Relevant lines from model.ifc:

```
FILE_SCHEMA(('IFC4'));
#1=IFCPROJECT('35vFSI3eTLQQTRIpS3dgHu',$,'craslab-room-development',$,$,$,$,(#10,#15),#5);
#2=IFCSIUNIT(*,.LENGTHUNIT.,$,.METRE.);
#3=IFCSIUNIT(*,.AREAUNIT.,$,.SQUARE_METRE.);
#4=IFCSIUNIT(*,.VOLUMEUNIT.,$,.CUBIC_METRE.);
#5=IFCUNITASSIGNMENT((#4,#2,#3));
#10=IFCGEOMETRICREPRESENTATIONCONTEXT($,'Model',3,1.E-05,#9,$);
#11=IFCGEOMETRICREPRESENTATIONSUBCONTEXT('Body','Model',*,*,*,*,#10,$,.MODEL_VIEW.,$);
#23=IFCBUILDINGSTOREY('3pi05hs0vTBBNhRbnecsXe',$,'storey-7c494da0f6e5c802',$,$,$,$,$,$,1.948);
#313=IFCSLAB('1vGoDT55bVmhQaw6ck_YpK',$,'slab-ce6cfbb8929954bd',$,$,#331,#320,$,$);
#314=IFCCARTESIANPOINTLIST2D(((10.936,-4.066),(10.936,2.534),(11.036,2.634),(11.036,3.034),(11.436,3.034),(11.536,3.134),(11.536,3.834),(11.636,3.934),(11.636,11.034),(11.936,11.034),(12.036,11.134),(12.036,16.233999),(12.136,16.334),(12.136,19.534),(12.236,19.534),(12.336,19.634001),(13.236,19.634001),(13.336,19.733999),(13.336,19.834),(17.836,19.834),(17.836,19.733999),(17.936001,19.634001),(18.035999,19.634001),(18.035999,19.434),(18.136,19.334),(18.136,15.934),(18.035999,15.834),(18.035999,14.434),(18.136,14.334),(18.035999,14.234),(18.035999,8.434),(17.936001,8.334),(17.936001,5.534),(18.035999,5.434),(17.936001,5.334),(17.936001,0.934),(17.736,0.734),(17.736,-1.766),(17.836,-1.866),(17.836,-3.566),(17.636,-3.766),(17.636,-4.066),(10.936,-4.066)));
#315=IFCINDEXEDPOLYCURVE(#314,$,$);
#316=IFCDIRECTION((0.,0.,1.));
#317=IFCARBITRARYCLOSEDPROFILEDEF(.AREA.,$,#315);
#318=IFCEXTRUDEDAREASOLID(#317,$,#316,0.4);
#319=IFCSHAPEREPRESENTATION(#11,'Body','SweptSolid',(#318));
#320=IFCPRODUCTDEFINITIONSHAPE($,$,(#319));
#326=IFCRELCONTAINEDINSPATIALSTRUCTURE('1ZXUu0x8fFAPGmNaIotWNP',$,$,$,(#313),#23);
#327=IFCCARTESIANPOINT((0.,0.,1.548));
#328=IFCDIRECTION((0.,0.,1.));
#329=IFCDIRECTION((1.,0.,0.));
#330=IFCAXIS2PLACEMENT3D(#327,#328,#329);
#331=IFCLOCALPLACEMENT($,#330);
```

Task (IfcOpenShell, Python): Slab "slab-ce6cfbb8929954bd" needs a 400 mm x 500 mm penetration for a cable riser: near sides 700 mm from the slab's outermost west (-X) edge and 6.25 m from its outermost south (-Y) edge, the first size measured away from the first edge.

```python
import numpy as np
import ifcopenshell
import ifcopenshell.api.feature
import ifcopenshell.api.geometry
import ifcopenshell.api.root
import ifcopenshell.geom
import ifcopenshell.util.placement
import ifcopenshell.util.representation
import ifcopenshell.util.shape
import ifcopenshell.util.unit

model = ifcopenshell.open("model.ifc")
unit_scale = ifcopenshell.util.unit.calculate_unit_scale(model)
settings = ifcopenshell.geom.settings()


def volume(element):
    """Net volume in cubic metres, openings subtracted."""
    shape = ifcopenshell.geom.create_shape(settings, element)
    return ifcopenshell.util.shape.get_volume(shape.geometry)


slab = model.by_guid("1vGoDT55bVmhQaw6ck_YpK")
before = volume(slab)

# Extent in the slab's own axes, in metres. The edges named are its -X and -Y sides.
slab_shape = ifcopenshell.geom.create_shape(settings, slab)
vertices = ifcopenshell.util.shape.get_vertices(slab_shape.geometry)
x_min, y_min, bottom = vertices.min(axis=0)
top = vertices[:, 2].max()

opening = ifcopenshell.api.root.create_entity(model, ifc_class="IfcOpeningElement", name="Cable riser opening", predefined_type="OPENING")
context = ifcopenshell.util.representation.get_context(model, "Model", "Body", "MODEL_VIEW")
width, depth = 0.4, 0.5
outline = [(0.0, 0.0), (width, 0.0), (width, depth), (0.0, depth), (0.0, 0.0)]
# Overshoot both faces by 50 mm so the cut is clean.
shape = ifcopenshell.api.geometry.add_slab_representation(
    model, context=context, depth=top - bottom + 0.1, polyline=outline
)
ifcopenshell.api.geometry.assign_representation(model, product=opening, representation=shape)

matrix = ifcopenshell.util.placement.get_local_placement(slab.ObjectPlacement)
matrix[:, 3] = matrix @ np.append(np.array([x_min + 0.7, y_min + 6.25, bottom - 0.05]) / unit_scale, 1.0)
ifcopenshell.api.geometry.edit_object_placement(model, product=opening, matrix=matrix, is_si=False)
ifcopenshell.api.feature.add_feature(model, feature=opening, element=slab)

after = volume(slab)

print(f"slab volume {before:.3f} -> {after:.3f} m3")

model.write("model_v2.ifc")
```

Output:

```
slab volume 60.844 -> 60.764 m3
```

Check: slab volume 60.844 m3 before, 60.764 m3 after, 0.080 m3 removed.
